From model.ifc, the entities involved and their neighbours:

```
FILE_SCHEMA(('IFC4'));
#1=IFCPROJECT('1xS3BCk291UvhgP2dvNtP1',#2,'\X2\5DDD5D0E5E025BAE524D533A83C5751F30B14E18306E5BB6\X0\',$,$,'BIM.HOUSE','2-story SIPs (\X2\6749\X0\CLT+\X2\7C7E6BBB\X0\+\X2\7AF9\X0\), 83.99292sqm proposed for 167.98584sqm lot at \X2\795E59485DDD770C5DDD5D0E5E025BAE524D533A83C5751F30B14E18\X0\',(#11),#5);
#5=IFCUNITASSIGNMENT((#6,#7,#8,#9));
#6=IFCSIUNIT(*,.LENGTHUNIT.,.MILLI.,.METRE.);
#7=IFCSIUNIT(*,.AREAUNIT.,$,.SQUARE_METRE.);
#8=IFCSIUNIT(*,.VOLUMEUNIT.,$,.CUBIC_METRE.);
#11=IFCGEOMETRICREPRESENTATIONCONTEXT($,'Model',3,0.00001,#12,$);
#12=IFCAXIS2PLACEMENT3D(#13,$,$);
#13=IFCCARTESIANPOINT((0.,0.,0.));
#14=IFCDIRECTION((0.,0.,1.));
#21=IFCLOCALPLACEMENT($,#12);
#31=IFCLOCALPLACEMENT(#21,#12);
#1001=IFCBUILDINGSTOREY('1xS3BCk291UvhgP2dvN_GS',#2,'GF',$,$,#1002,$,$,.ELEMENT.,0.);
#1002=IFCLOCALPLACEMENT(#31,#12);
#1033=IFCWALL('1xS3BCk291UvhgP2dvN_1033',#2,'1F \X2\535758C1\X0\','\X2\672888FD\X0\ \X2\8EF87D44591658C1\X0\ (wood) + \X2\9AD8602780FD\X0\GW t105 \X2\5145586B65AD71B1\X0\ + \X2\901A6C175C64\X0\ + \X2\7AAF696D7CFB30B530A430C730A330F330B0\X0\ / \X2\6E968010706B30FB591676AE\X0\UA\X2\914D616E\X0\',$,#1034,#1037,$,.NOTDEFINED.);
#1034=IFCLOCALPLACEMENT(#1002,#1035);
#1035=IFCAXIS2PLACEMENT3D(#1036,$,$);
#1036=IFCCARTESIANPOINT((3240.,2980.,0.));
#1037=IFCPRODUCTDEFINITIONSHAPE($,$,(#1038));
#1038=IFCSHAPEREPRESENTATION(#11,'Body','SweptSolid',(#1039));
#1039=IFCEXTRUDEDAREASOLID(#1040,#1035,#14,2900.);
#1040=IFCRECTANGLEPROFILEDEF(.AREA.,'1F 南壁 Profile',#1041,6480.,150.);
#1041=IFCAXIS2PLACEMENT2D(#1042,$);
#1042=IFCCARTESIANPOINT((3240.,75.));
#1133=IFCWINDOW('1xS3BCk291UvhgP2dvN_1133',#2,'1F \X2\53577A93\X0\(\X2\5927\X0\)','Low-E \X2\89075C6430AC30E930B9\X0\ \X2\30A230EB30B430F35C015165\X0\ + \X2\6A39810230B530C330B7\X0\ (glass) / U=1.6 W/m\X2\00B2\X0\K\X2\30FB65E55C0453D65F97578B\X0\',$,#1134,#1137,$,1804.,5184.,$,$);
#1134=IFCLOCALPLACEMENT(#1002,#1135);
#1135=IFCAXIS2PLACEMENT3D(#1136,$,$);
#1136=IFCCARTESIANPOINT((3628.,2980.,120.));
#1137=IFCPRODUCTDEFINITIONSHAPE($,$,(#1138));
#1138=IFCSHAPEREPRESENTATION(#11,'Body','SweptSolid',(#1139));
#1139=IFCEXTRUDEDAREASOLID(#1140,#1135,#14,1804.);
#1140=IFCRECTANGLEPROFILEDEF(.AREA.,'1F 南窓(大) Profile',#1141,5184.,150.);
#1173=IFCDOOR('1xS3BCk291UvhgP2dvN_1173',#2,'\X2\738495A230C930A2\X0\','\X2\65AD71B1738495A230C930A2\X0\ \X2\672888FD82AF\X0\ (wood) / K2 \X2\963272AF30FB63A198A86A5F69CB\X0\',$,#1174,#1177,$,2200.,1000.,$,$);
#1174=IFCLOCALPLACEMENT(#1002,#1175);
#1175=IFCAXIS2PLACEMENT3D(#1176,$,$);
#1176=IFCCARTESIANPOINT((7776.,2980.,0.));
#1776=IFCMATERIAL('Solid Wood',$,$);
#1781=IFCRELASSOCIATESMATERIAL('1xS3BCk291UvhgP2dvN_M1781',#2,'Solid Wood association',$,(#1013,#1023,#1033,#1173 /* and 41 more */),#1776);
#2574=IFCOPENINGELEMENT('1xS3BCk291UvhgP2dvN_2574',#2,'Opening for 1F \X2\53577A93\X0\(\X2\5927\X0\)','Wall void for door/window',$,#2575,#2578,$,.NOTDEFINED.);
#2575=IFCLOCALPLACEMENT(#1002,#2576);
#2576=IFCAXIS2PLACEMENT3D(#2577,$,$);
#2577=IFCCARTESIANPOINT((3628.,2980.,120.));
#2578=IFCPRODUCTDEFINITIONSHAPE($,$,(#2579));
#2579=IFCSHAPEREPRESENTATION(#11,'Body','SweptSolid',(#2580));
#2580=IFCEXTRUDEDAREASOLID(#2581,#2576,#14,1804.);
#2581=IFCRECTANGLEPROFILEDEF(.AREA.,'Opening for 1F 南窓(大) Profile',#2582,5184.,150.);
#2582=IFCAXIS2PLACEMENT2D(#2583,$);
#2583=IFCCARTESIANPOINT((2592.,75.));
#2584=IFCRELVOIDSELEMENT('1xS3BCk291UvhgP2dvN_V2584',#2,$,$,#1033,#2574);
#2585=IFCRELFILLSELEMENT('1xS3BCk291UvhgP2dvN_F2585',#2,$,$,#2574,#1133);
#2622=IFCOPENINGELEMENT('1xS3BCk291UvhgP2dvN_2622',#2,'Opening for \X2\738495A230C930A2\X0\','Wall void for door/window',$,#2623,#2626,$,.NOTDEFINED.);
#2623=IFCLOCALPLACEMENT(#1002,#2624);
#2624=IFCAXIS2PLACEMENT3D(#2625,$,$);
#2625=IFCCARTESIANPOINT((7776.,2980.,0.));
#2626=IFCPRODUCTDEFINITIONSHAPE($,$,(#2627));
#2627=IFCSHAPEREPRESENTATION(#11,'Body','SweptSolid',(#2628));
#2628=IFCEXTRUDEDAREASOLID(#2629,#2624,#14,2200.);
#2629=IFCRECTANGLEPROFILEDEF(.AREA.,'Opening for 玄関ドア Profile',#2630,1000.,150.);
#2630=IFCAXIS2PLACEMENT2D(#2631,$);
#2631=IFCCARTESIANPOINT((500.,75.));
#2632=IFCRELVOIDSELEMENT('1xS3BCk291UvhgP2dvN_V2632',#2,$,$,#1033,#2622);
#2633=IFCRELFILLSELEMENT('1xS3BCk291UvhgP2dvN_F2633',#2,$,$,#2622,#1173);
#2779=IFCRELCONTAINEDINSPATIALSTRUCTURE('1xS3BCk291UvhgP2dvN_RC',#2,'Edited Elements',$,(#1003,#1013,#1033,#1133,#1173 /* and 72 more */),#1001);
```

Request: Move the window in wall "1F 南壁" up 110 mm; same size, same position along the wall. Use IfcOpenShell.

```python
import numpy as np
import ifcopenshell
import ifcopenshell.api.geometry
import ifcopenshell.util.placement
import ifcopenshell.util.unit

model = ifcopenshell.open("model.ifc")
unit_scale = ifcopenshell.util.unit.calculate_unit_scale(model)

window = model.by_guid("1xS3BCk291UvhgP2dvN_1133")
opening = window.FillsVoids[0].RelatingOpeningElement
dz = 0.11 / unit_scale

shift = np.array([0.0, 0.0, dz])
# The window is not placed relative to its opening, so move both.
for product in (opening, window):
    matrix = ifcopenshell.util.placement.get_local_placement(product.ObjectPlacement)
    matrix[:3, 3] += shift
    ifcopenshell.api.geometry.edit_object_placement(model, product=product, matrix=matrix, is_si=False)

print(f"moved by {dz * unit_scale:+.3f} m")

model.write("model_rev.ifc")
```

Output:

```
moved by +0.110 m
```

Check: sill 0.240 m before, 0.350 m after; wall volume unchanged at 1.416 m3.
